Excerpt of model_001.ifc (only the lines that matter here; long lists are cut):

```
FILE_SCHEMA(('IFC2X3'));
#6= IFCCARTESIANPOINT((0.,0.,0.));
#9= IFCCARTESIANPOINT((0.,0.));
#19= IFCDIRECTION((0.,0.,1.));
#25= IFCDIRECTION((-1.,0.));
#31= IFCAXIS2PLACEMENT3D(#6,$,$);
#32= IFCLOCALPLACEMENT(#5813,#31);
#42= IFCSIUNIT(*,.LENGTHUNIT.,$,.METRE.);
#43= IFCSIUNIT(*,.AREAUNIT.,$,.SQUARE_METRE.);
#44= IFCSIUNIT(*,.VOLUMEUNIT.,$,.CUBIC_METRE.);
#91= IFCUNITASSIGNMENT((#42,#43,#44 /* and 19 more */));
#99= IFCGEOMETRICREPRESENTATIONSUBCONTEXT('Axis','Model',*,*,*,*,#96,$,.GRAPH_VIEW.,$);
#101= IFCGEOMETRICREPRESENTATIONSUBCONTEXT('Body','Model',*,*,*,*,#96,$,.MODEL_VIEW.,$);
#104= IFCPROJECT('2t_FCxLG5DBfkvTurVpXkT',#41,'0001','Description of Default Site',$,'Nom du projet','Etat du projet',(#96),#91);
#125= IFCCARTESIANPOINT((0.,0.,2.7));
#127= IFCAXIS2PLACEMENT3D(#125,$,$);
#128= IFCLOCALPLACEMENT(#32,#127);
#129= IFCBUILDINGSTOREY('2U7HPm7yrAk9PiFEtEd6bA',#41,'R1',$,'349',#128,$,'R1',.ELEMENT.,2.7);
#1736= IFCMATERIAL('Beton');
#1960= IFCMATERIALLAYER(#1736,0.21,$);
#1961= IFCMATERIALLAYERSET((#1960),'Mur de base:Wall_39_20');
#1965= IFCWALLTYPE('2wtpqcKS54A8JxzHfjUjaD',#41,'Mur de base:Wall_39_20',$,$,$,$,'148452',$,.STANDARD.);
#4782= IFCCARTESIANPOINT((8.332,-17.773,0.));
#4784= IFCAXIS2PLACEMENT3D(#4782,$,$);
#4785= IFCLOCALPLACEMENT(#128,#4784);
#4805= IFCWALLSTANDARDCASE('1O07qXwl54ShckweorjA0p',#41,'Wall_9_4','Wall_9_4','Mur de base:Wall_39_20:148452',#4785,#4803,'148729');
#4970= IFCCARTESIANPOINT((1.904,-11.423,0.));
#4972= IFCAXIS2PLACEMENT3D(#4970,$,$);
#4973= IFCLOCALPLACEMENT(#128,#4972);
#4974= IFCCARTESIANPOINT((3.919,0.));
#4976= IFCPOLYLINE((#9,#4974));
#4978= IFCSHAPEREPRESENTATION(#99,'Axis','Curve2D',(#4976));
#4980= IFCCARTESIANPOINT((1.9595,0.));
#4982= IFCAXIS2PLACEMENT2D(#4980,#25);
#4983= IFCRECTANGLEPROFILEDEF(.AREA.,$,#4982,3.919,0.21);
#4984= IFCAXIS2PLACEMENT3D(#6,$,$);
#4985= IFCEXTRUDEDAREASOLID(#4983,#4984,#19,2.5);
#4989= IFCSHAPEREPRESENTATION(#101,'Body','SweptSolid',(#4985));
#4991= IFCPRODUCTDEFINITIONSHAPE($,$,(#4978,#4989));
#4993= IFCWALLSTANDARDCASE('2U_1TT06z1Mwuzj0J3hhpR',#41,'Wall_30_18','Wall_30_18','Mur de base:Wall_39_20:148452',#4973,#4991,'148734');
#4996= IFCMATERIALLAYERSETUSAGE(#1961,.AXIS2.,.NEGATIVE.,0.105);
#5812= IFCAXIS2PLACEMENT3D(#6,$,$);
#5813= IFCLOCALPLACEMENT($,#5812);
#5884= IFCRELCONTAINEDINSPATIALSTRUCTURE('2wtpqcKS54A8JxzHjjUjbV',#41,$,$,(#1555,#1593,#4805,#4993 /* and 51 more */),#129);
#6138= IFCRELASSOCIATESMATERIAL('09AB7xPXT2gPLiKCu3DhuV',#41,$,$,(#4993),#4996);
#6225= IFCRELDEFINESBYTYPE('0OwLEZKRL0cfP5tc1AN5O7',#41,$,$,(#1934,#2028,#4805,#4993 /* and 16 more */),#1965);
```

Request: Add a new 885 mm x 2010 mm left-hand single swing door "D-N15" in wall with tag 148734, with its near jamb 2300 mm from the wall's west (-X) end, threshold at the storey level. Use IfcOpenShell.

```python
import numpy as np
import ifcopenshell
import ifcopenshell.api.feature
import ifcopenshell.api.geometry
import ifcopenshell.api.root
import ifcopenshell.api.spatial
import ifcopenshell.api.type
import ifcopenshell.geom
import ifcopenshell.util.element
import ifcopenshell.util.placement
import ifcopenshell.util.representation
import ifcopenshell.util.shape
import ifcopenshell.util.unit

model = ifcopenshell.open("model_001.ifc")
unit_scale = ifcopenshell.util.unit.calculate_unit_scale(model)
settings = ifcopenshell.geom.settings()


def volume(element):
    """Net volume in cubic metres, openings subtracted."""
    shape = ifcopenshell.geom.create_shape(settings, element)
    return ifcopenshell.util.shape.get_volume(shape.geometry)


wall = model.by_guid("2U_1TT06z1Mwuzj0J3hhpR")
storey = ifcopenshell.util.element.get_container(wall, ifc_class="IfcBuildingStorey")
context = ifcopenshell.util.representation.get_context(model, "Model", "Body", "MODEL_VIEW")
before = volume(wall)

width, height, from_end, sill = 0.885, 2.01, 2.3, 0.0  # metres

# The wall runs along its own X axis, and the end named is its -X end.
wall_shape = ifcopenshell.geom.create_shape(settings, wall)
x, y, z = ifcopenshell.util.shape.get_vertices(wall_shape.geometry).T
start = x.min() + from_end
face, thickness = float(y.min()), float(y.max() - y.min())
wall_matrix = ifcopenshell.util.placement.get_local_placement(wall.ObjectPlacement)
level = ifcopenshell.util.placement.get_local_placement(storey.ObjectPlacement)[2, 3]


def in_wall(x, y):
    """Placement at x, y metres in the wall's axes, at sill height."""
    matrix = wall_matrix.copy()
    matrix[:, 3] = wall_matrix @ np.array([x / unit_scale, y / unit_scale, 0.0, 1.0])
    matrix[2, 3] = level + sill / unit_scale
    return matrix


# Opening: a box that overshoots both wall faces by 50 mm.
opening = ifcopenshell.api.root.create_entity(model, ifc_class="IfcOpeningElement")
box = ifcopenshell.api.geometry.add_wall_representation(
    model, context=context, length=width, height=height, thickness=thickness + 0.1
)
ifcopenshell.api.geometry.assign_representation(model, product=opening, representation=box)
ifcopenshell.api.geometry.edit_object_placement(model, product=opening, matrix=in_wall(start, face - 0.05), is_si=False)
ifcopenshell.api.feature.add_feature(model, feature=opening, element=wall)

door = ifcopenshell.api.root.create_entity(model, ifc_class="IfcDoor", name="D-N15")
door.OverallWidth, door.OverallHeight = width / unit_scale, height / unit_scale
body = ifcopenshell.api.geometry.add_door_representation(
    model,
    context=context,
    overall_width=door.OverallWidth,
    overall_height=door.OverallHeight,
    operation_type="SINGLE_SWING_LEFT",
    lining_properties={"LiningDepth": thickness / unit_scale, "ThresholdDepth": thickness / unit_scale},
)
ifcopenshell.api.geometry.assign_representation(model, product=door, representation=body)
ifcopenshell.api.spatial.assign_container(model, products=[door], relating_structure=storey)
fills = ifcopenshell.api.feature.add_filling(model, opening=opening, element=door)
fills.OwnerHistory = door.OwnerHistory  # required in IFC2X3

# IFC2X3 keeps the operation on the door style.
style = ifcopenshell.api.root.create_entity(model, ifc_class="IfcDoorStyle", name="D-N15")
style.OperationType, style.ConstructionType = "SINGLE_SWING_LEFT", "NOTDEFINED"
style.ParameterTakesPrecedence = style.Sizeable = False
ifcopenshell.api.type.assign_type(model, related_objects=[door], relating_type=style)

# The lining spans the wall, so the door starts at the wall face.
ifcopenshell.api.geometry.edit_object_placement(model, product=door, matrix=in_wall(start, face), is_si=False)

after = volume(wall)

print(f"wall volume {before:.3f} -> {after:.3f} m3")

model.write("model_001_v2.ifc")
```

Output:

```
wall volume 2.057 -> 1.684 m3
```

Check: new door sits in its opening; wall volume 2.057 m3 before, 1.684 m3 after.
